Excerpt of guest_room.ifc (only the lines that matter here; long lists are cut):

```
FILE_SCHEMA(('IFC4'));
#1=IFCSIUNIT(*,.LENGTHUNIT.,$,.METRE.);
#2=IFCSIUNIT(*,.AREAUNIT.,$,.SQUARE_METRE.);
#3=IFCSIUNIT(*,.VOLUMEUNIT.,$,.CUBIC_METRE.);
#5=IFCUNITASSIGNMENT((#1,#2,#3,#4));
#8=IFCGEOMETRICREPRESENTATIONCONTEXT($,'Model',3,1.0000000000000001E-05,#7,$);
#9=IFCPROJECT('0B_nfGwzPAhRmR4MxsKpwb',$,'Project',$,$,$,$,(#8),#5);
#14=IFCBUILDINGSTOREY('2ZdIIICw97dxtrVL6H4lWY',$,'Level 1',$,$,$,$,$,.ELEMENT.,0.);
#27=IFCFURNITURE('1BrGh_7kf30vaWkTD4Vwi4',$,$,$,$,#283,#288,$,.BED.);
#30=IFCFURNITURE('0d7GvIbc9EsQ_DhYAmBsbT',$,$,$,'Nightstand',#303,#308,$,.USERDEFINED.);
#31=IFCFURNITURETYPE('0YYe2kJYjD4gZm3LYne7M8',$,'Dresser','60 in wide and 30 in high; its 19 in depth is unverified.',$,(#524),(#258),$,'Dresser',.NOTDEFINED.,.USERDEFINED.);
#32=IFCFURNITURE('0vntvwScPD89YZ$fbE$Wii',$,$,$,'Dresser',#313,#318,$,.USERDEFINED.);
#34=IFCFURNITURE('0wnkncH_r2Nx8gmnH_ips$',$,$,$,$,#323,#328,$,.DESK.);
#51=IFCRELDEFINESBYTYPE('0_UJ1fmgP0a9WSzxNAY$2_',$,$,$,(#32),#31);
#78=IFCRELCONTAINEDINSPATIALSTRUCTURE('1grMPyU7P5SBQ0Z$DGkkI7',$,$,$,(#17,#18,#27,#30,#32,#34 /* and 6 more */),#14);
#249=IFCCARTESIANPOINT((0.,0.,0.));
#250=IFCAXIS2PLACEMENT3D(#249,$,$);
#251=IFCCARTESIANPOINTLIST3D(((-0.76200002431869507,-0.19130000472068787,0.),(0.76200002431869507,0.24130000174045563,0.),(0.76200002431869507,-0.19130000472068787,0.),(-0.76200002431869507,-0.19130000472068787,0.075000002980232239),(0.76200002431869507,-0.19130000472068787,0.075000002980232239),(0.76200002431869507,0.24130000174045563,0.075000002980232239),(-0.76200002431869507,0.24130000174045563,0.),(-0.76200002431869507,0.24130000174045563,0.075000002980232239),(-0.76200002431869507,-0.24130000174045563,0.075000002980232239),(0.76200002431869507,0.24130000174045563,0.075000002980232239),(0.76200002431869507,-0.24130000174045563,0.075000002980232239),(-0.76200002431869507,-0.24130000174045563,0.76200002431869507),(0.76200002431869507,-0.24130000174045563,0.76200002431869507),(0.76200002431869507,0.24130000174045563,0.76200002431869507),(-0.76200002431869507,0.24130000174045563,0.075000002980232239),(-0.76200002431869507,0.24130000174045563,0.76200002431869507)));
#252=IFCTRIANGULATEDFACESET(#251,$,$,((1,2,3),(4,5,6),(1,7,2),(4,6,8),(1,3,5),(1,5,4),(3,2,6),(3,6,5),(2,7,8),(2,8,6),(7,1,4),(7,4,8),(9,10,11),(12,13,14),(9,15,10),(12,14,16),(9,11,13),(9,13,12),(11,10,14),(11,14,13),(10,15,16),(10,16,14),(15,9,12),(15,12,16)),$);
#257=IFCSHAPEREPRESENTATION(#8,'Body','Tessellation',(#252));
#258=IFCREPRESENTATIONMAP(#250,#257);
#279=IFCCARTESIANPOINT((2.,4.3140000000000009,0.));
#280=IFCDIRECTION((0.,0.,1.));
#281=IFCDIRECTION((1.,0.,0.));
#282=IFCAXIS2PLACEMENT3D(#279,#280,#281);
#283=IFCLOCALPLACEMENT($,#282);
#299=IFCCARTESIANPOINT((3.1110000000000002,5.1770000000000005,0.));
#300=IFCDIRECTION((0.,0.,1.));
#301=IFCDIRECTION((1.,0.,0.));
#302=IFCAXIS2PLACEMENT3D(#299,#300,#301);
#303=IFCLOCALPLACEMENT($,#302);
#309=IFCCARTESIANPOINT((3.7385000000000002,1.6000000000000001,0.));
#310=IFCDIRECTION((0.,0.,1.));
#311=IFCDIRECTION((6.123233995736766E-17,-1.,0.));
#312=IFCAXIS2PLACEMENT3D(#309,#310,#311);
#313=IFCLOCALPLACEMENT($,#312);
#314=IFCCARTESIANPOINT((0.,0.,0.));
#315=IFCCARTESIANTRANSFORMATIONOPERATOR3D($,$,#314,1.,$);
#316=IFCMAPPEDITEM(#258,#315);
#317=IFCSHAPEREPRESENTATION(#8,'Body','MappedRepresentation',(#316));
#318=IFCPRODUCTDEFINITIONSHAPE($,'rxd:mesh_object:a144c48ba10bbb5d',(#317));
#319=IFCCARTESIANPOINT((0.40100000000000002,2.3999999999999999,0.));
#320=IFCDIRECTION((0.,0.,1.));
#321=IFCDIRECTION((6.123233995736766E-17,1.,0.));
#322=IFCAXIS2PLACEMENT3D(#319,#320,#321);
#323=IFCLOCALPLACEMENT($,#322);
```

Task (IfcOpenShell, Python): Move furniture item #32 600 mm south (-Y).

```python
import ifcopenshell
import ifcopenshell.api.geometry
import ifcopenshell.util.placement
import ifcopenshell.util.unit

model = ifcopenshell.open("guest_room.ifc")
unit_scale = ifcopenshell.util.unit.calculate_unit_scale(model)

item = model.by_id(32)
matrix = ifcopenshell.util.placement.get_local_placement(item.ObjectPlacement)
matrix[1, 3] -= 0.6 / unit_scale
ifcopenshell.api.geometry.edit_object_placement(model, product=item, matrix=matrix, is_si=False)

print(ifcopenshell.util.placement.get_local_placement(item.ObjectPlacement).round(3) + 0.0)

model.write("guest_room_rev.ifc")
```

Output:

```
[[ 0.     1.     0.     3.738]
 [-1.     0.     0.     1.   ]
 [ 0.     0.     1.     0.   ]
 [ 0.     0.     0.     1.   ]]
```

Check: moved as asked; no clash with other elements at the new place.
